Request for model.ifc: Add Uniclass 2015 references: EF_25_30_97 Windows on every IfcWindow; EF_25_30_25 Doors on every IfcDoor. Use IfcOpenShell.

First a look at what the model holds.

```python
import ifcopenshell

model = ifcopenshell.open("model.ifc")
print(model.schema)
print("classifications:", [c.Name for c in model.by_type("IfcClassification")])
for ifc_class in ("IfcDoor", "IfcRoof", "IfcStair", "IfcWall", "IfcWindow"):
    print(ifc_class, len(model.by_type(ifc_class)))
```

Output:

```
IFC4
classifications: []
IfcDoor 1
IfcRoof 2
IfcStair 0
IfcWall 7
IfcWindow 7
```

```python
import ifcopenshell
import ifcopenshell.api.classification

model = ifcopenshell.open("model.ifc")

system = ifcopenshell.api.classification.add_classification(model, classification="Uniclass 2015")

codes = {
    "IfcWindow": ("EF_25_30_97", "Windows"),
    "IfcDoor": ("EF_25_30_25", "Doors"),
}
for ifc_class, (code, name) in codes.items():
    products = model.by_type(ifc_class)
    ifcopenshell.api.classification.add_reference(
        model, products=products, classification=system, identification=code, name=name
    )
    print(code, len(products))

model.write("model-out.ifc")
```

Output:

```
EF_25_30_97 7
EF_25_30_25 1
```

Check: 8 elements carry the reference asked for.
